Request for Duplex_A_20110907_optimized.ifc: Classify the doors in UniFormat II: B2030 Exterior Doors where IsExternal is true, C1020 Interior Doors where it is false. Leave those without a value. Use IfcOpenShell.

First a look at what the model holds.

```python
import ifcopenshell
import ifcopenshell.util.element

model = ifcopenshell.open("Duplex_A_20110907_optimized.ifc")
print(model.schema)
print("classifications:", [c.Name for c in model.by_type("IfcClassification")])
values = [ifcopenshell.util.element.get_pset(e, "Pset_DoorCommon", "IsExternal") for e in model.by_type("IfcDoor")]
for value in (True, False, None):
    print("IsExternal", value, values.count(value))
```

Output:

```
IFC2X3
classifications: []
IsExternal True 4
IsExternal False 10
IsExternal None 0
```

```python
import ifcopenshell
import ifcopenshell.api.classification
import ifcopenshell.util.element

model = ifcopenshell.open("Duplex_A_20110907_optimized.ifc")

# IFC2X3 requires Source and Edition and has no link from the project to the system.
system = model.create_entity("IfcClassification", Source="ASTM", Edition="E1557", Name="UniFormat II")

doors = model.by_type("IfcDoor")
external = {e: ifcopenshell.util.element.get_pset(e, "Pset_DoorCommon", "IsExternal") for e in doors}
for flag, code, name in ((True, "B2030", "Exterior Doors"), (False, "C1020", "Interior Doors")):
    products = [e for e in doors if external[e] is flag]
    ifcopenshell.api.classification.add_reference(
        model, products=products, classification=system, identification=code, name=name
    )
    print(code, len(products))

model.write("Duplex_A_20110907_optimized_edited.ifc")
```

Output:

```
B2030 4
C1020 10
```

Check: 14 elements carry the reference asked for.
